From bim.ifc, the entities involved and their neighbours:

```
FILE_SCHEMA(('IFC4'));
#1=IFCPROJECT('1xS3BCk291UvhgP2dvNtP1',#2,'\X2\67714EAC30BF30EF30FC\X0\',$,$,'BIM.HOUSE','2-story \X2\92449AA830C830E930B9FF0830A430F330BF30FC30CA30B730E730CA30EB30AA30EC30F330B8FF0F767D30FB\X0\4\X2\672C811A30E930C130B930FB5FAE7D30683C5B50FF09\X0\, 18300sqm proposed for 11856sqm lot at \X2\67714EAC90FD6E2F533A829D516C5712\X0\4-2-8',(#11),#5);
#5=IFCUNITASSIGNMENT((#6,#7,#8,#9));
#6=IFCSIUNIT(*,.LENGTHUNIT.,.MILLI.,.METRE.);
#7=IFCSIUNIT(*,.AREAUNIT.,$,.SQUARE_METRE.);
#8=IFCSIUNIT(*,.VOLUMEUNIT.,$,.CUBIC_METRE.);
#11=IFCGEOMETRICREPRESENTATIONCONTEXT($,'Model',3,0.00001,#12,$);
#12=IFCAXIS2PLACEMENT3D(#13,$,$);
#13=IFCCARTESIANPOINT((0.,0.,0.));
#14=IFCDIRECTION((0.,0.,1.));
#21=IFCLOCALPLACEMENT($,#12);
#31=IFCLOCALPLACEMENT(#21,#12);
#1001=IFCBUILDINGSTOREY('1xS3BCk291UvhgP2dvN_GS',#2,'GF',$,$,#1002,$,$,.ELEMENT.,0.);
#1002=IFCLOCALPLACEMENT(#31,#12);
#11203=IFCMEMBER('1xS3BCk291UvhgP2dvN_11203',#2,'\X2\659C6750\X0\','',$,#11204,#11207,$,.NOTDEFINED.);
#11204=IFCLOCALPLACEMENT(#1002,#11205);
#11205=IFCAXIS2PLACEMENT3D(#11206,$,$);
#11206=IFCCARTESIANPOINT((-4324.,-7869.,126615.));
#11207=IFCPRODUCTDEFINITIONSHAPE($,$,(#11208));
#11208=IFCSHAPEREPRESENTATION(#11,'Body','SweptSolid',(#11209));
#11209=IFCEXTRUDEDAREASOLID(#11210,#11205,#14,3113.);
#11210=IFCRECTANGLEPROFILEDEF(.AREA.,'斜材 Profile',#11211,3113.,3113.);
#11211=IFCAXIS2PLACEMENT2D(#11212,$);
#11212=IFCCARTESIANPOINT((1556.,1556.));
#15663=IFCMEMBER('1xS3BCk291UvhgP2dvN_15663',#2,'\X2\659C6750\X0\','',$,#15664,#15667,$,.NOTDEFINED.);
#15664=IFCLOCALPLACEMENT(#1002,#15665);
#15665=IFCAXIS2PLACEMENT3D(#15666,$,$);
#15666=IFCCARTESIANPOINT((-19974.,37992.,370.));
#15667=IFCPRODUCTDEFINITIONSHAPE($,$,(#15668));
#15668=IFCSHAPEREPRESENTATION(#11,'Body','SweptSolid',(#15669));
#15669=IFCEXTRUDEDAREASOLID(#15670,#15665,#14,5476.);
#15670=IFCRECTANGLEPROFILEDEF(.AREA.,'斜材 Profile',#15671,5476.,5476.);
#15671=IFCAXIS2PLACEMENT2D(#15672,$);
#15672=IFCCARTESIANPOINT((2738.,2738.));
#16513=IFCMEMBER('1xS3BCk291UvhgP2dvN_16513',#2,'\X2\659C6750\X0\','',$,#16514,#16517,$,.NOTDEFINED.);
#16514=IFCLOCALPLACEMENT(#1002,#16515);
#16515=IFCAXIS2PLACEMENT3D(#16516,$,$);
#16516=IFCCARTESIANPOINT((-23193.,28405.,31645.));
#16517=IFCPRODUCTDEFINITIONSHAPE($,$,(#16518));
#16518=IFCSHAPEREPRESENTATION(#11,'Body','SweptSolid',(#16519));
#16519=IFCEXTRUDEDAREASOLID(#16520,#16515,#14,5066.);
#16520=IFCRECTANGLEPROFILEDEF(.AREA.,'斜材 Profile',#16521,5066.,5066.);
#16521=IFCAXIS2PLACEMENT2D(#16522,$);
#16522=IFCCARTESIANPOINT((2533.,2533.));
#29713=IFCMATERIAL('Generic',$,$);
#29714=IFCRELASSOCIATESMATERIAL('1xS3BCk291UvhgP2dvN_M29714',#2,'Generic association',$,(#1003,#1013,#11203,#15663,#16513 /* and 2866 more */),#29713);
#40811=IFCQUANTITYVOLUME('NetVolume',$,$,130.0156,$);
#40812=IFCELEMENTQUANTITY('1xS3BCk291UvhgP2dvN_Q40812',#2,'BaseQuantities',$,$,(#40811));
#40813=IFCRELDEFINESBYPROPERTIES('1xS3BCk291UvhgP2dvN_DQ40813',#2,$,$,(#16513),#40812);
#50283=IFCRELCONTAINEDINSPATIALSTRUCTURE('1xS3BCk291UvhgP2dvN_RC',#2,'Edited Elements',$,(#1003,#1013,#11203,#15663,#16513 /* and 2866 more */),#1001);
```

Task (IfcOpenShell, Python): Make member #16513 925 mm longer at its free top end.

```python
import ifcopenshell
import ifcopenshell.api.pset
import ifcopenshell.util.element

model = ifcopenshell.open("bim.ifc")

member = model.by_guid("1xS3BCk291UvhgP2dvN_16513")
change = 925.0

# The extrusion runs towards the end named, so only its depth changes.
body = next(r for r in member.Representation.Representations if r.RepresentationIdentifier == "Body")
solid = body.Items[0]
old_length = solid.Depth
solid.Depth += change

# Update the stored length and volume.
qto = model.by_id(ifcopenshell.util.element.get_pset(member, "BaseQuantities", should_inherit=False)["id"])
ifcopenshell.api.pset.edit_qto(model, qto=qto, properties={
    "NetVolume": ifcopenshell.util.element.get_pset(member, "BaseQuantities", "NetVolume") * solid.Depth / old_length,
})

print(f"length {old_length:g} -> {solid.Depth:g}")

model.write("bim_edited.ifc")
```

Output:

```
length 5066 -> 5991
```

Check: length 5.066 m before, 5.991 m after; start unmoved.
